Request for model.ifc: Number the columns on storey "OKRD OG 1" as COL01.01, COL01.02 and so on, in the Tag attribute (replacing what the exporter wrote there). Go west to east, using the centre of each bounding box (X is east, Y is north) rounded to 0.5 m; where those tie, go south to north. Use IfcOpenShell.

First a look at what the model holds.

```python
import ifcopenshell
import ifcopenshell.util.element
import ifcopenshell.util.placement

model = ifcopenshell.open("model.ifc")
print(model.schema)
storey = next(s for s in model.by_type("IfcBuildingStorey") if s.Name == "OKRD OG 1")
columns = [e for e in ifcopenshell.util.element.get_decomposition(storey) if e.is_a("IfcColumn")]
for e in sorted(columns, key=lambda e: e.id()):
    origin = ifcopenshell.util.placement.get_local_placement(e.ObjectPlacement)[:3, 3]
    print(e.id(), e.Tag, e.Name, origin.round(2) + 0.0, sep=" | ")
```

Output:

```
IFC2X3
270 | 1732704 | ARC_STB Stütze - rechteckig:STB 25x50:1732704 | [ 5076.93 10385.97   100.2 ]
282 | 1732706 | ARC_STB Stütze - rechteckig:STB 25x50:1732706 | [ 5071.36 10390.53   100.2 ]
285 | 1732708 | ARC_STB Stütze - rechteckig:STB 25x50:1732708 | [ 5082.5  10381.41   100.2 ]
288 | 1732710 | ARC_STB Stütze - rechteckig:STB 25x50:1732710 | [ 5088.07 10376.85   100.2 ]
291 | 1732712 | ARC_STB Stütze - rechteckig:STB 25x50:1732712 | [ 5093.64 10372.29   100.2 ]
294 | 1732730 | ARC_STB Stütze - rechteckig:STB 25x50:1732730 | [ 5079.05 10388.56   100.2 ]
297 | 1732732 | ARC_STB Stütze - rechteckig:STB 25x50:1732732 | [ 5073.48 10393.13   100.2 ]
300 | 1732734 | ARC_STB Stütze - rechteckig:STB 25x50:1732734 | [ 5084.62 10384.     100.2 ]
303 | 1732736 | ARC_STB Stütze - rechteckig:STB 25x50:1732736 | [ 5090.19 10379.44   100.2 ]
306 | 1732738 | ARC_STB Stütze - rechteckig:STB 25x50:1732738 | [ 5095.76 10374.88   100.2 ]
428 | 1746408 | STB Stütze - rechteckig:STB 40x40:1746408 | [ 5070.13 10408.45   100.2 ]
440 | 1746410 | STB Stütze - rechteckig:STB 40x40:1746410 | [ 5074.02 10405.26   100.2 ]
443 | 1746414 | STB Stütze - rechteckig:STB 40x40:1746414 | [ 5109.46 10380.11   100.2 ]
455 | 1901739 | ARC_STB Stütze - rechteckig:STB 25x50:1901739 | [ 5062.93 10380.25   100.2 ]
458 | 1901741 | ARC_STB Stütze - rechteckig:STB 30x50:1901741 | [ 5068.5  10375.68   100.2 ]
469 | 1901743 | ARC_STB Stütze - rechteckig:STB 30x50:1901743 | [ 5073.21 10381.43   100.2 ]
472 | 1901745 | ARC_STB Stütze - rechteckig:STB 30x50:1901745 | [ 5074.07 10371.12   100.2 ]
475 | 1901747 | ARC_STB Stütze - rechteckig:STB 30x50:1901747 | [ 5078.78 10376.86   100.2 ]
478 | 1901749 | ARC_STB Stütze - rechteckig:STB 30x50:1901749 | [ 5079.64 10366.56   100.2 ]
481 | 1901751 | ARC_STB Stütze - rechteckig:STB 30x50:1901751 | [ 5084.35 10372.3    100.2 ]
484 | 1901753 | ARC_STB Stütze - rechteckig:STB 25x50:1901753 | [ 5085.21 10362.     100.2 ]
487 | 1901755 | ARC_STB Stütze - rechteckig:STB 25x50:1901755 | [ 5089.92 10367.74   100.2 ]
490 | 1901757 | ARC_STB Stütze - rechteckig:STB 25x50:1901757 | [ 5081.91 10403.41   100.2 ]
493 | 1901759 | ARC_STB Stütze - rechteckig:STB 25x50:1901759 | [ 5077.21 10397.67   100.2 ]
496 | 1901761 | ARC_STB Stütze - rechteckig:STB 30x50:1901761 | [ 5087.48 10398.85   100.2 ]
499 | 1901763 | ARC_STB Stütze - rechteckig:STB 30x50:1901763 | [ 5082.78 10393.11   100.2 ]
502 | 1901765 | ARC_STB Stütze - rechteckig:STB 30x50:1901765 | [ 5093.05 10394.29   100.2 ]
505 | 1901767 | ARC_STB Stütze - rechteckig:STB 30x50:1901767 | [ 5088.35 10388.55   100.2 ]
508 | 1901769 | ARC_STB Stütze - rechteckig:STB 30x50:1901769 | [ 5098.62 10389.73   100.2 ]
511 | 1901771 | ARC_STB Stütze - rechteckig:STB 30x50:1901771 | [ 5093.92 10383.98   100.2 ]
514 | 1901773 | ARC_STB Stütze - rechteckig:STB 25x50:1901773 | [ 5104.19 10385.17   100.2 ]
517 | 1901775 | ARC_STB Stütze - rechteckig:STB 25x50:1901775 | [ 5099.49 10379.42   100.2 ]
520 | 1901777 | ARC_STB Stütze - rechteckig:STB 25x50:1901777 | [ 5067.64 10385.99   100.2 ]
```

```python
import ifcopenshell
import ifcopenshell.geom
import ifcopenshell.util.element
import ifcopenshell.util.shape

model = ifcopenshell.open("model.ifc")
settings = ifcopenshell.geom.settings()
settings.set("use-world-coords", True)


def centre(element):
    shape = ifcopenshell.geom.create_shape(settings, element)
    return ifcopenshell.util.shape.get_bbox_centroid(shape.geometry)


storey = next(s for s in model.by_type("IfcBuildingStorey") if s.Name == "OKRD OG 1")
columns = [e for e in ifcopenshell.util.element.get_decomposition(storey) if e.is_a("IfcColumn")]

# Insertion points can sit at a corner or the storey origin, so sort by the geometry (in metres).
centres = {e: centre(e) for e in columns}
columns.sort(key=lambda e: (round(centres[e][0] / 0.5), centres[e][1]))

for i, e in enumerate(columns, start=1):
    number = f"COL01.{i:02d}"
    e.Tag = number
    print(e.id(), number)

model.write("model-out.ifc")
```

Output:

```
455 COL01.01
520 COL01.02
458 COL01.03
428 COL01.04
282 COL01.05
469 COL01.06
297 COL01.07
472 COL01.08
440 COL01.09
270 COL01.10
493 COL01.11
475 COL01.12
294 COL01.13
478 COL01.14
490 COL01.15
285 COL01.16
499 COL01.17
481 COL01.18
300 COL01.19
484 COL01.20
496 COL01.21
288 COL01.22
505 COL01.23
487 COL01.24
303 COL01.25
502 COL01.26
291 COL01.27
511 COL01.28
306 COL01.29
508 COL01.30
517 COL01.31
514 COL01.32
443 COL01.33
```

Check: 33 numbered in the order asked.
